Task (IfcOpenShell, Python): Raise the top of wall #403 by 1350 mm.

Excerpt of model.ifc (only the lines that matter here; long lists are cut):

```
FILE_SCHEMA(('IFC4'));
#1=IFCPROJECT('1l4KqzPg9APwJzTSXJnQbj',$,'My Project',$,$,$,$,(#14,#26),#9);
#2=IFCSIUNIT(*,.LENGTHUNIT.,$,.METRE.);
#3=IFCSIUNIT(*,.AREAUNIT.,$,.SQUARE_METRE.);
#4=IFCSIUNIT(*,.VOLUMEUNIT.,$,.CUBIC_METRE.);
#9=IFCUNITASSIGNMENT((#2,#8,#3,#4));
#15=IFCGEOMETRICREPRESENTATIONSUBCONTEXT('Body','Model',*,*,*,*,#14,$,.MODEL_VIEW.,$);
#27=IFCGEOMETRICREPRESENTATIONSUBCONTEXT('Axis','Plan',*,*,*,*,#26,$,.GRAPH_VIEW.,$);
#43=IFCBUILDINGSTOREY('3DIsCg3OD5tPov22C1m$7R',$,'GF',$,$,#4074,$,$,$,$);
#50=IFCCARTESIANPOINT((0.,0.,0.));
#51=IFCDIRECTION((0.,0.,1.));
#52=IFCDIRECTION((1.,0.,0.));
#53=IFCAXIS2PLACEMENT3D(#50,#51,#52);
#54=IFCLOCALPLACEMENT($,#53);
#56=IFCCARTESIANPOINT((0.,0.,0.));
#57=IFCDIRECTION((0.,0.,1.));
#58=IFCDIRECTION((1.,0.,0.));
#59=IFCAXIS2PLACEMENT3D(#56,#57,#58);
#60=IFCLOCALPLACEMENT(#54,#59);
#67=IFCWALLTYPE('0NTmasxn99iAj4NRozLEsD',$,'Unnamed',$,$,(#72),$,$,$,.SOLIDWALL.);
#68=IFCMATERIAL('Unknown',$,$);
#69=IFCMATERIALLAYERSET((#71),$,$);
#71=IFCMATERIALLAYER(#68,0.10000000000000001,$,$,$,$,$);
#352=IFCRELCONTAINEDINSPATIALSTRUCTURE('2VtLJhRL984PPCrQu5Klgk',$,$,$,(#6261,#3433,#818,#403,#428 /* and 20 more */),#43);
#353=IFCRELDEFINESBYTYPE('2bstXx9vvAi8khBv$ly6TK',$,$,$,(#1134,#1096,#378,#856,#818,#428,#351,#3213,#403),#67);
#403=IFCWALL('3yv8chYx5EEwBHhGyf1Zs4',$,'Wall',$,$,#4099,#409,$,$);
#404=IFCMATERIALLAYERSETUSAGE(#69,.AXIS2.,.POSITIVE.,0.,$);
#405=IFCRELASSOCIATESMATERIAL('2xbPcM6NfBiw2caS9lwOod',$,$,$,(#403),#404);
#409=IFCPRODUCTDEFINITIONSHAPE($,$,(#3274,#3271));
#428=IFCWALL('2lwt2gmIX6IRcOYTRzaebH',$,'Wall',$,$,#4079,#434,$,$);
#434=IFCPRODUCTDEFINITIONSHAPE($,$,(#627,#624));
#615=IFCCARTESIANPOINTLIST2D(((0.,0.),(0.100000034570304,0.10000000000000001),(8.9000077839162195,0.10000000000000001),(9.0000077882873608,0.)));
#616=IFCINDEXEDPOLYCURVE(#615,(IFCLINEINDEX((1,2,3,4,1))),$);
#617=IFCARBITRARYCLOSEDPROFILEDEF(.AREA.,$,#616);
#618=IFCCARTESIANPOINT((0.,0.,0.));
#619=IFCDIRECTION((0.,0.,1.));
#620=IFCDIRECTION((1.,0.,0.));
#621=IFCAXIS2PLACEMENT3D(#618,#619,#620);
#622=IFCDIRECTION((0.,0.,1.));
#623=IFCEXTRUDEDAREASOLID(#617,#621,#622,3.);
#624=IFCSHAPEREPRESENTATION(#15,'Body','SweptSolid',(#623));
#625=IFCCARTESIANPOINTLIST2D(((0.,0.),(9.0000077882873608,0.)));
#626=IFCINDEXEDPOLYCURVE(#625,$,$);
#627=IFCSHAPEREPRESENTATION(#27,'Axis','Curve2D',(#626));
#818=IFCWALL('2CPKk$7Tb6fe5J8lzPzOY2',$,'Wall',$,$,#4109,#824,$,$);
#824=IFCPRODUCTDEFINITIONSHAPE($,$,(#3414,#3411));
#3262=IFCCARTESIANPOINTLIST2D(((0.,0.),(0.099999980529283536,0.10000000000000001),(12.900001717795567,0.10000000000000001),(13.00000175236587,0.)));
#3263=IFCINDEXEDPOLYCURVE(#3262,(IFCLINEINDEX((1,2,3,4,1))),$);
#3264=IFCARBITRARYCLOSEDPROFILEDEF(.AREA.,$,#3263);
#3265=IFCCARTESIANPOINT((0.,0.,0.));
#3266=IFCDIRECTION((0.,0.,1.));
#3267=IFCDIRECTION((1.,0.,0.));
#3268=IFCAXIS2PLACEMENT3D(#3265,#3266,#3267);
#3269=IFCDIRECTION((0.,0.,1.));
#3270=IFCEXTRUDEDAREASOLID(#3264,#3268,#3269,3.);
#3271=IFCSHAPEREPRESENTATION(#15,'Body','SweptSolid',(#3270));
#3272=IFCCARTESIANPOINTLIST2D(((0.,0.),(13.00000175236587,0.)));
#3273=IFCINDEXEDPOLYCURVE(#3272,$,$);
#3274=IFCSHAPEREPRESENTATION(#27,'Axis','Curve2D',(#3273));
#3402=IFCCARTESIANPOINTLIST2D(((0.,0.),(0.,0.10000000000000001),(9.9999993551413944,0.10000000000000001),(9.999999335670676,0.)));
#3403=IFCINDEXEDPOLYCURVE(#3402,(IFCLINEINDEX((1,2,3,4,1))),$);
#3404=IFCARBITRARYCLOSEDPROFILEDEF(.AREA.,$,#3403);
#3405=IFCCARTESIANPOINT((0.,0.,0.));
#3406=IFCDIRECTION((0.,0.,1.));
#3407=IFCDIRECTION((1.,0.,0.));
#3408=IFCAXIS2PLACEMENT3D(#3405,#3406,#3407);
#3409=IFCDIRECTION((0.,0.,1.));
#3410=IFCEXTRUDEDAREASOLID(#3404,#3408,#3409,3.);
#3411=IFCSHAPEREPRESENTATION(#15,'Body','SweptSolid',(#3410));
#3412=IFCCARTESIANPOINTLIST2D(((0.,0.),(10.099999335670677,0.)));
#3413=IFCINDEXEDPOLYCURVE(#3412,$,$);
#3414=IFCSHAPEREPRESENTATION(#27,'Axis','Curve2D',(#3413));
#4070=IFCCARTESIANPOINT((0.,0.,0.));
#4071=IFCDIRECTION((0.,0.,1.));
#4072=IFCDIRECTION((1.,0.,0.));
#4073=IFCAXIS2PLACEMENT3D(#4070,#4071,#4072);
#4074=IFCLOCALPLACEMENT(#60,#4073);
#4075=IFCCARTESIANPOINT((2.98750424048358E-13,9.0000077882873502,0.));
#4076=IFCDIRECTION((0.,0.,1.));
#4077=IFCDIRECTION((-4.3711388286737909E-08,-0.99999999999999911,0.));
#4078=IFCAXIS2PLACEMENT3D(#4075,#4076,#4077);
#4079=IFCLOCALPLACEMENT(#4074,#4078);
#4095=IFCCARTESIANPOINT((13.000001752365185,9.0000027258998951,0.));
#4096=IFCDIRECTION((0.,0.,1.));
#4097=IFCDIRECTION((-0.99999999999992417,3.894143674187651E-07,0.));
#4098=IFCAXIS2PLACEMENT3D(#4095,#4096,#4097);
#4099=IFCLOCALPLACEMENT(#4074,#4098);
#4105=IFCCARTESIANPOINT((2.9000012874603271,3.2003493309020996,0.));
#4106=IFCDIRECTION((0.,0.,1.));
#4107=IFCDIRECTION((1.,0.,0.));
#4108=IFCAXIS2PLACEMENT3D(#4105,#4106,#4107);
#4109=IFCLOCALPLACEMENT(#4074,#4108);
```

```python
import ifcopenshell
import ifcopenshell.geom
import ifcopenshell.util.representation
import ifcopenshell.util.shape

model = ifcopenshell.open("model.ifc")
settings = ifcopenshell.geom.settings()


def volume(element):
    """Net volume in cubic metres, openings subtracted."""
    shape = ifcopenshell.geom.create_shape(settings, element)
    return ifcopenshell.util.shape.get_volume(shape.geometry)


wall = model.by_guid("3yv8chYx5EEwBHhGyf1Zs4")
before = volume(wall)

body = ifcopenshell.util.representation.get_representation(wall, "Model", "Body")
solid = body.Items[0]
old_height = solid.Depth
solid.Depth += 1.35
after = volume(wall)

print(f"height {old_height:g} -> {solid.Depth:g}, volume {before:.3f} -> {after:.3f} m3")

model.write("model_updated.ifc")
```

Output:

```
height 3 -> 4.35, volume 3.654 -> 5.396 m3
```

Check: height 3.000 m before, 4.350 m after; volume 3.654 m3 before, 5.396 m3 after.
